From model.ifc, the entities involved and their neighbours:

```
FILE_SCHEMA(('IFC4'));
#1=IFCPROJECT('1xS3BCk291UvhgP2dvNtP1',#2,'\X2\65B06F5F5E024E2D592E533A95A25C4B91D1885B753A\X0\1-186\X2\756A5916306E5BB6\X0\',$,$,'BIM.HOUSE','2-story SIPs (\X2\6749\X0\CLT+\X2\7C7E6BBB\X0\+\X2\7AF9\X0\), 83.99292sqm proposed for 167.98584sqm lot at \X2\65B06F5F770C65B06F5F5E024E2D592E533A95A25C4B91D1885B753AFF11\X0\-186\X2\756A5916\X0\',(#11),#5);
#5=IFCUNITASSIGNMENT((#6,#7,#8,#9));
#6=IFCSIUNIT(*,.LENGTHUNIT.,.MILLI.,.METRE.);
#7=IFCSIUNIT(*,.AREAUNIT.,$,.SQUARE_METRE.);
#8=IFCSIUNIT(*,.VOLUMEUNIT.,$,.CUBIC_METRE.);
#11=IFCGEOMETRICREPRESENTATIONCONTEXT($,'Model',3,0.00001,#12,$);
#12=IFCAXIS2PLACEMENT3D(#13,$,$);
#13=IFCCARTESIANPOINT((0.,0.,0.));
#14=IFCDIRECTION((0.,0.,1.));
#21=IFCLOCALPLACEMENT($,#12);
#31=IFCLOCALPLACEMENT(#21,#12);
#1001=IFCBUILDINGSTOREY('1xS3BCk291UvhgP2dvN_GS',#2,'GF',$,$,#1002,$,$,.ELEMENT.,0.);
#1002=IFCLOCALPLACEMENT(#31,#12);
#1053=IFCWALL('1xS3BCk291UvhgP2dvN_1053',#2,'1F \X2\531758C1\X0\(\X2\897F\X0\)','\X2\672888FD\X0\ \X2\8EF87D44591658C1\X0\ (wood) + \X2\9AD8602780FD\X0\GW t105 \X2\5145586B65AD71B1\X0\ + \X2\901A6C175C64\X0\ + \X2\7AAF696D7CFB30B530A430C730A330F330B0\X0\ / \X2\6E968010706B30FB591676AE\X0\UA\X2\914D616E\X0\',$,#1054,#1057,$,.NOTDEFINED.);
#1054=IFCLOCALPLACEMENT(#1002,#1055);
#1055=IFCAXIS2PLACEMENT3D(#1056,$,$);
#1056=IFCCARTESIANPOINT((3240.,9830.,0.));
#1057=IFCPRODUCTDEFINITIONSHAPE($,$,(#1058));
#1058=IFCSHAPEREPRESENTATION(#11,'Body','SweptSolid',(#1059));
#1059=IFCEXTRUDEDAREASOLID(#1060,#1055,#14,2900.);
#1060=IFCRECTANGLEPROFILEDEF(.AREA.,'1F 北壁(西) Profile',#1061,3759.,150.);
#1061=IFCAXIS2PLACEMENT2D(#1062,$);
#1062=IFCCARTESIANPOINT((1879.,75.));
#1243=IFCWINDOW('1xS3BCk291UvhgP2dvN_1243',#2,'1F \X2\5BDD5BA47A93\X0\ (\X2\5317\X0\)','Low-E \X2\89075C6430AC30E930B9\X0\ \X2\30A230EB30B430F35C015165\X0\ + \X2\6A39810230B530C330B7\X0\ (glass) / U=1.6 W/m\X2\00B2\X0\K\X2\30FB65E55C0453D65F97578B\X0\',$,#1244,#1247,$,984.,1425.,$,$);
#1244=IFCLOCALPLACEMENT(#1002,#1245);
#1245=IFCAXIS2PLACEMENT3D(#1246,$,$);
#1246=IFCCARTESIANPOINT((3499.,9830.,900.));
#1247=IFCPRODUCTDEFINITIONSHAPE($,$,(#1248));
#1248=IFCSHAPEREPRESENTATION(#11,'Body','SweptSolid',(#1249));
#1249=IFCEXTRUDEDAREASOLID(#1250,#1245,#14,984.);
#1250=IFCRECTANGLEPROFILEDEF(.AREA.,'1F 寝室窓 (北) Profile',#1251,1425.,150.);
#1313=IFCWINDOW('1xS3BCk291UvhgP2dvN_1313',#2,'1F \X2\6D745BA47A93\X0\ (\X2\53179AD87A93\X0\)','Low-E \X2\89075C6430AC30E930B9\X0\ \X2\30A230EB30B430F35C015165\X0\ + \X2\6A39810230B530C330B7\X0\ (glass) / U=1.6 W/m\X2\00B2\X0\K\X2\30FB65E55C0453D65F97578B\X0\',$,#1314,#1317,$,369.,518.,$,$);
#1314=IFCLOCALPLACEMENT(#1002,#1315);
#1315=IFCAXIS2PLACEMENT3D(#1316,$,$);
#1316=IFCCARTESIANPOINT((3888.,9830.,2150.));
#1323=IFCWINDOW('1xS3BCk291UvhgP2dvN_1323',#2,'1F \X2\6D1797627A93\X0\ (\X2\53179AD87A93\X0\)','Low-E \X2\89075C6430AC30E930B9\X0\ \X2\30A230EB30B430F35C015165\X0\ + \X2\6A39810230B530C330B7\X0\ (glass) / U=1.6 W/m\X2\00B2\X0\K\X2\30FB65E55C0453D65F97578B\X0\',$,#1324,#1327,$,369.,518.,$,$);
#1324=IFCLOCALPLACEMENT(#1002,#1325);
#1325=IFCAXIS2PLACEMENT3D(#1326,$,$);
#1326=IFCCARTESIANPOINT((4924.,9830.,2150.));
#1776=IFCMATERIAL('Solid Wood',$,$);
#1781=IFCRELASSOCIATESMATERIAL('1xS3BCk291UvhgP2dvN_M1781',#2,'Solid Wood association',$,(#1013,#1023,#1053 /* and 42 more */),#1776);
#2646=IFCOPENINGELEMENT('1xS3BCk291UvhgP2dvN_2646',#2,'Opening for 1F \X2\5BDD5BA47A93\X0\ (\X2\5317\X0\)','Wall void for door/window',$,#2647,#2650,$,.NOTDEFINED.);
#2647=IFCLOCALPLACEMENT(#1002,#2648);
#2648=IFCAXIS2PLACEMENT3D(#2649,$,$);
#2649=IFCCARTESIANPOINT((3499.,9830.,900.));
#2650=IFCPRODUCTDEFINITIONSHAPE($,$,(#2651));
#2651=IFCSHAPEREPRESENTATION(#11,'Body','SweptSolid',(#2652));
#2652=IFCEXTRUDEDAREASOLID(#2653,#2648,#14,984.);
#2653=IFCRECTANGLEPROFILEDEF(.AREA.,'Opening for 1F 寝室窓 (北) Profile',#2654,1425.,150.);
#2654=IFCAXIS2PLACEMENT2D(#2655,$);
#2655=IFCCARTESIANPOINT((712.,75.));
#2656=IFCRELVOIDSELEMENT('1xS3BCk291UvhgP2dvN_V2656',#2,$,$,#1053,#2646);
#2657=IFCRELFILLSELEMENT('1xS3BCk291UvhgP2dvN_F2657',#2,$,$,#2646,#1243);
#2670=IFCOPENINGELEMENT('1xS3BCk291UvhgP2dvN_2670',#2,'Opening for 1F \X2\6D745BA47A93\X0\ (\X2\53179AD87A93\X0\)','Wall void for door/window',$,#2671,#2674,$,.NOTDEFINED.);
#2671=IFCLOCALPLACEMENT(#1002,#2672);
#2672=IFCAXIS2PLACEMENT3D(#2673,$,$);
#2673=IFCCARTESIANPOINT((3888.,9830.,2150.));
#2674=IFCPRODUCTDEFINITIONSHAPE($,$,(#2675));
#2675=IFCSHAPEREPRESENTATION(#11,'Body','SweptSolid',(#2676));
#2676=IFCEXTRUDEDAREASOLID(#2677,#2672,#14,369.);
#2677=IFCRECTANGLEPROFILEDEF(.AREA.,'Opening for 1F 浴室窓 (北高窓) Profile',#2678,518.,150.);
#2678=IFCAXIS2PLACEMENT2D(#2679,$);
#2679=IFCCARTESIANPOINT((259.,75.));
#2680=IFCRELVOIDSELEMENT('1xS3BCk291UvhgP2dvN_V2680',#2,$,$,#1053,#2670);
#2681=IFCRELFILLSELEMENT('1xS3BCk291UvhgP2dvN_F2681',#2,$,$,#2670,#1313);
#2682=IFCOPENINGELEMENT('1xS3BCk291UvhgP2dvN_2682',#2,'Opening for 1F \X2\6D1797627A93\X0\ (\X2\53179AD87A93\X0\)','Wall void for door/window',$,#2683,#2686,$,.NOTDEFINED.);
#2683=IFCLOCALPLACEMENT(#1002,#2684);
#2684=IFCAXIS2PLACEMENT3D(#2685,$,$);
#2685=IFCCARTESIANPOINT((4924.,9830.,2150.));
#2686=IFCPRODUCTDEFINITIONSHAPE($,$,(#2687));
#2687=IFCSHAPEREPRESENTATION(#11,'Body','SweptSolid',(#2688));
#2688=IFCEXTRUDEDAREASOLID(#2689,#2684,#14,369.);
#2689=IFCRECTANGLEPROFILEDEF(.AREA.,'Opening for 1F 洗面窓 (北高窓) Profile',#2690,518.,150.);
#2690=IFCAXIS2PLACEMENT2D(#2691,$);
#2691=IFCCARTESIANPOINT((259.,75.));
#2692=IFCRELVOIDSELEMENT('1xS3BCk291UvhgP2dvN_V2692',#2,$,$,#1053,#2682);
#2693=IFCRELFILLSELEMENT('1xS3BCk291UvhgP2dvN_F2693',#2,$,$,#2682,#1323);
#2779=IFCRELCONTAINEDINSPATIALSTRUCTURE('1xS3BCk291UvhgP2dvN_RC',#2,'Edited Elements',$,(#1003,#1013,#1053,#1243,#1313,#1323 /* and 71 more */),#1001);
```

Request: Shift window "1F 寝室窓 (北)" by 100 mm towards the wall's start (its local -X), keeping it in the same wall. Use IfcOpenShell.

```python
import ifcopenshell
import ifcopenshell.api.geometry
import ifcopenshell.util.placement

model = ifcopenshell.open("model.ifc")

window = model.by_guid("1xS3BCk291UvhgP2dvN_1243")
opening = window.FillsVoids[0].RelatingOpeningElement
wall = opening.VoidsElements[0].RelatingBuildingElement

wall_matrix = ifcopenshell.util.placement.get_local_placement(wall.ObjectPlacement)
shift = wall_matrix[:3, 0] * -100.0
before = ifcopenshell.util.placement.get_local_placement(window.ObjectPlacement)[:3, 3].copy()

# The window is not placed relative to its opening, so move both.
for product in (opening, window):
    matrix = ifcopenshell.util.placement.get_local_placement(product.ObjectPlacement)
    matrix[:3, 3] += shift
    ifcopenshell.api.geometry.edit_object_placement(model, product=product, matrix=matrix, is_si=False)

after = ifcopenshell.util.placement.get_local_placement(window.ObjectPlacement)[:3, 3]
print("window moved by", (after - before).round(3) + 0.0)

model.write("model_updated.ifc")
```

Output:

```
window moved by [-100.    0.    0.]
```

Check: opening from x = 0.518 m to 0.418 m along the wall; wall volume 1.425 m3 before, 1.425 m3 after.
